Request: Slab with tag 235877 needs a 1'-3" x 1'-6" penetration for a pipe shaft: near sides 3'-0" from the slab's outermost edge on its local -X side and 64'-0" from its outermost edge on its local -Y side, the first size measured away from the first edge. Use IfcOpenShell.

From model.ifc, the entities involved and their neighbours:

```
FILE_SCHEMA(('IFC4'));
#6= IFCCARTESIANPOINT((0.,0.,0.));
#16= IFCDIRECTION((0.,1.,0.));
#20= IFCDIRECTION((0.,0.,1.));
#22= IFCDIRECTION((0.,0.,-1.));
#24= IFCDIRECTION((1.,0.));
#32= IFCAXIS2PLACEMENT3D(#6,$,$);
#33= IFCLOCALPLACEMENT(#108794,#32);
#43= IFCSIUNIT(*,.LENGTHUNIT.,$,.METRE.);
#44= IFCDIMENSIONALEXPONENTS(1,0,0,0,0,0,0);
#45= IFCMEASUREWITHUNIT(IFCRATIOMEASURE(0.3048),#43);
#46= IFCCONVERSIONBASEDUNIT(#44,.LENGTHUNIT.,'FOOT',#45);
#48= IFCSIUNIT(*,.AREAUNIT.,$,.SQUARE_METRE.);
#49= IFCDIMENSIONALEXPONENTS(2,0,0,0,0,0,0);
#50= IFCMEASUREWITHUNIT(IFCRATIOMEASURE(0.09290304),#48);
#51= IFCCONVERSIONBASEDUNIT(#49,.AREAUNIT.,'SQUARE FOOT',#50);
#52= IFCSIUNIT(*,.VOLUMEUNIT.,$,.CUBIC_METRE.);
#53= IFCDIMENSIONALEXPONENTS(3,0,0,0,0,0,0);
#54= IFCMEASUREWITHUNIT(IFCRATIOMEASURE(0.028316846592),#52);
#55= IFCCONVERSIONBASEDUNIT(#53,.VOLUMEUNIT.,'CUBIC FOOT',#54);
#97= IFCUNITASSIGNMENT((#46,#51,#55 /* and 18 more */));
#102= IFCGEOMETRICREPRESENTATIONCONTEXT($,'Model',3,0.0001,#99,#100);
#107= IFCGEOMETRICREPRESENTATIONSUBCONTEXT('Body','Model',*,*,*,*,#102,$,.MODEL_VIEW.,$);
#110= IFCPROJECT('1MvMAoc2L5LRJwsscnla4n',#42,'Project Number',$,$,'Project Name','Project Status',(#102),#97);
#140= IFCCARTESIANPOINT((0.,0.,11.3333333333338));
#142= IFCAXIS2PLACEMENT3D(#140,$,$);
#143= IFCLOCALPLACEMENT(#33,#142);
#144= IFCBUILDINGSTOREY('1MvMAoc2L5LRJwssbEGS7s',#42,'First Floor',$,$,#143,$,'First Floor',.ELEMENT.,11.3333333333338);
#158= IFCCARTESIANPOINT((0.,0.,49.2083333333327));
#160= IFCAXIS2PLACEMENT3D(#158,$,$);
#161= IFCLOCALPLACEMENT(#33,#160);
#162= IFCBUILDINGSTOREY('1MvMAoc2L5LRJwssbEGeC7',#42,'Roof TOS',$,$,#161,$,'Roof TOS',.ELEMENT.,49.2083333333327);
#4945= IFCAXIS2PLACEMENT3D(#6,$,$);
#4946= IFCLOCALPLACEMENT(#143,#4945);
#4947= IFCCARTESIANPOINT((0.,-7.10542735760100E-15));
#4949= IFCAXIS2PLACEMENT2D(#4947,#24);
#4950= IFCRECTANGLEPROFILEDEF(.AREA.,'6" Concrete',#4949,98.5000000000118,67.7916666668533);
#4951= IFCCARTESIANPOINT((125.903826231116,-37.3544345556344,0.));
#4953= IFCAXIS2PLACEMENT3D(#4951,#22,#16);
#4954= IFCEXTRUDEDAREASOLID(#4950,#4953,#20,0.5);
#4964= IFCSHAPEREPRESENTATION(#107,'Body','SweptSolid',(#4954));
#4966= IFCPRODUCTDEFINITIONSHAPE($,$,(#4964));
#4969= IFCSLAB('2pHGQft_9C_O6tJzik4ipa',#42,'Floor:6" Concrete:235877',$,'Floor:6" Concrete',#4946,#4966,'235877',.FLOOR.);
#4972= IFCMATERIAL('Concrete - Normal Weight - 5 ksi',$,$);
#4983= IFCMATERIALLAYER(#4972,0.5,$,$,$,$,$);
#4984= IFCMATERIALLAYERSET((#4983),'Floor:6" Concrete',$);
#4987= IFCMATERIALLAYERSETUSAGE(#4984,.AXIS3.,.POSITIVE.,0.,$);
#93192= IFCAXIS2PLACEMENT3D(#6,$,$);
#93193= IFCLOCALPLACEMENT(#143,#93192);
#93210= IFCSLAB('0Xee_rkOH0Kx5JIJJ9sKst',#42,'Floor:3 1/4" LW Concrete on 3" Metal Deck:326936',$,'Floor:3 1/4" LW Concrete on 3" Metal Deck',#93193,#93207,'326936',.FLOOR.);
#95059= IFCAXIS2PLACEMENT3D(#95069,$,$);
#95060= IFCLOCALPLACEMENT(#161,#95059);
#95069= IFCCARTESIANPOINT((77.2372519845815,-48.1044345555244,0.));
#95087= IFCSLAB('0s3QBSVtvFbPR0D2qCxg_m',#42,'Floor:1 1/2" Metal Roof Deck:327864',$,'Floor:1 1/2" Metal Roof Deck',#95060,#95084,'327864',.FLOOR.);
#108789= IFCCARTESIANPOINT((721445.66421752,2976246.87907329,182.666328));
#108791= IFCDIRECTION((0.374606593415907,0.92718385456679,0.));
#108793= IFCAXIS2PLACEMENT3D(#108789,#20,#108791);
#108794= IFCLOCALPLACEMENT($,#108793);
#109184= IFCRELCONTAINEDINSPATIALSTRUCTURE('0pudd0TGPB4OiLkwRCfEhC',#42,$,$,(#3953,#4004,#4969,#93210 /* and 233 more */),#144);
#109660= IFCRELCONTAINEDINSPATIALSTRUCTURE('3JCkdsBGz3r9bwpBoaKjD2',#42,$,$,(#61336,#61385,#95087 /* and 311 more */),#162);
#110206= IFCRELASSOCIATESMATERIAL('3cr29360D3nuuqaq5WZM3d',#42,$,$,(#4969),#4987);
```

```python
import numpy as np
import ifcopenshell
import ifcopenshell.api.feature
import ifcopenshell.api.geometry
import ifcopenshell.api.root
import ifcopenshell.geom
import ifcopenshell.util.placement
import ifcopenshell.util.representation
import ifcopenshell.util.shape
import ifcopenshell.util.unit

model = ifcopenshell.open("model.ifc")
unit_scale = ifcopenshell.util.unit.calculate_unit_scale(model)
settings = ifcopenshell.geom.settings()


def volume(element):
    """Net volume in cubic metres, openings subtracted."""
    shape = ifcopenshell.geom.create_shape(settings, element)
    return ifcopenshell.util.shape.get_volume(shape.geometry)


slab = model.by_id(4969)
before = volume(slab)

# Extent in the slab's own axes, in metres. The edges named are its -X and -Y sides.
slab_shape = ifcopenshell.geom.create_shape(settings, slab)
vertices = ifcopenshell.util.shape.get_vertices(slab_shape.geometry)
x_min, y_min, bottom = vertices.min(axis=0)
top = vertices[:, 2].max()

opening = ifcopenshell.api.root.create_entity(model, ifc_class="IfcOpeningElement", name="Pipe shaft opening", predefined_type="OPENING")
context = ifcopenshell.util.representation.get_context(model, "Model", "Body", "MODEL_VIEW")
width, depth = 0.381, 0.4572
outline = [(0.0, 0.0), (width, 0.0), (width, depth), (0.0, depth), (0.0, 0.0)]
# Overshoot both faces by 50 mm so the cut is clean.
shape = ifcopenshell.api.geometry.add_slab_representation(
    model, context=context, depth=top - bottom + 0.1, polyline=outline
)
ifcopenshell.api.geometry.assign_representation(model, product=opening, representation=shape)

matrix = ifcopenshell.util.placement.get_local_placement(slab.ObjectPlacement)
matrix[:, 3] = matrix @ np.append(np.array([x_min + 0.9144, y_min + 19.5072, bottom - 0.05]) / unit_scale, 1.0)
ifcopenshell.api.geometry.edit_object_placement(model, product=opening, matrix=matrix, is_si=False)
ifcopenshell.api.feature.add_feature(model, feature=opening, element=slab)

after = volume(slab)

print(f"slab volume {before:.3f} -> {after:.3f} m3")

model.write("model_updated.ifc")
```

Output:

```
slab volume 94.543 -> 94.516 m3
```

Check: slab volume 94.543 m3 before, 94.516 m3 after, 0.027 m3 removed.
